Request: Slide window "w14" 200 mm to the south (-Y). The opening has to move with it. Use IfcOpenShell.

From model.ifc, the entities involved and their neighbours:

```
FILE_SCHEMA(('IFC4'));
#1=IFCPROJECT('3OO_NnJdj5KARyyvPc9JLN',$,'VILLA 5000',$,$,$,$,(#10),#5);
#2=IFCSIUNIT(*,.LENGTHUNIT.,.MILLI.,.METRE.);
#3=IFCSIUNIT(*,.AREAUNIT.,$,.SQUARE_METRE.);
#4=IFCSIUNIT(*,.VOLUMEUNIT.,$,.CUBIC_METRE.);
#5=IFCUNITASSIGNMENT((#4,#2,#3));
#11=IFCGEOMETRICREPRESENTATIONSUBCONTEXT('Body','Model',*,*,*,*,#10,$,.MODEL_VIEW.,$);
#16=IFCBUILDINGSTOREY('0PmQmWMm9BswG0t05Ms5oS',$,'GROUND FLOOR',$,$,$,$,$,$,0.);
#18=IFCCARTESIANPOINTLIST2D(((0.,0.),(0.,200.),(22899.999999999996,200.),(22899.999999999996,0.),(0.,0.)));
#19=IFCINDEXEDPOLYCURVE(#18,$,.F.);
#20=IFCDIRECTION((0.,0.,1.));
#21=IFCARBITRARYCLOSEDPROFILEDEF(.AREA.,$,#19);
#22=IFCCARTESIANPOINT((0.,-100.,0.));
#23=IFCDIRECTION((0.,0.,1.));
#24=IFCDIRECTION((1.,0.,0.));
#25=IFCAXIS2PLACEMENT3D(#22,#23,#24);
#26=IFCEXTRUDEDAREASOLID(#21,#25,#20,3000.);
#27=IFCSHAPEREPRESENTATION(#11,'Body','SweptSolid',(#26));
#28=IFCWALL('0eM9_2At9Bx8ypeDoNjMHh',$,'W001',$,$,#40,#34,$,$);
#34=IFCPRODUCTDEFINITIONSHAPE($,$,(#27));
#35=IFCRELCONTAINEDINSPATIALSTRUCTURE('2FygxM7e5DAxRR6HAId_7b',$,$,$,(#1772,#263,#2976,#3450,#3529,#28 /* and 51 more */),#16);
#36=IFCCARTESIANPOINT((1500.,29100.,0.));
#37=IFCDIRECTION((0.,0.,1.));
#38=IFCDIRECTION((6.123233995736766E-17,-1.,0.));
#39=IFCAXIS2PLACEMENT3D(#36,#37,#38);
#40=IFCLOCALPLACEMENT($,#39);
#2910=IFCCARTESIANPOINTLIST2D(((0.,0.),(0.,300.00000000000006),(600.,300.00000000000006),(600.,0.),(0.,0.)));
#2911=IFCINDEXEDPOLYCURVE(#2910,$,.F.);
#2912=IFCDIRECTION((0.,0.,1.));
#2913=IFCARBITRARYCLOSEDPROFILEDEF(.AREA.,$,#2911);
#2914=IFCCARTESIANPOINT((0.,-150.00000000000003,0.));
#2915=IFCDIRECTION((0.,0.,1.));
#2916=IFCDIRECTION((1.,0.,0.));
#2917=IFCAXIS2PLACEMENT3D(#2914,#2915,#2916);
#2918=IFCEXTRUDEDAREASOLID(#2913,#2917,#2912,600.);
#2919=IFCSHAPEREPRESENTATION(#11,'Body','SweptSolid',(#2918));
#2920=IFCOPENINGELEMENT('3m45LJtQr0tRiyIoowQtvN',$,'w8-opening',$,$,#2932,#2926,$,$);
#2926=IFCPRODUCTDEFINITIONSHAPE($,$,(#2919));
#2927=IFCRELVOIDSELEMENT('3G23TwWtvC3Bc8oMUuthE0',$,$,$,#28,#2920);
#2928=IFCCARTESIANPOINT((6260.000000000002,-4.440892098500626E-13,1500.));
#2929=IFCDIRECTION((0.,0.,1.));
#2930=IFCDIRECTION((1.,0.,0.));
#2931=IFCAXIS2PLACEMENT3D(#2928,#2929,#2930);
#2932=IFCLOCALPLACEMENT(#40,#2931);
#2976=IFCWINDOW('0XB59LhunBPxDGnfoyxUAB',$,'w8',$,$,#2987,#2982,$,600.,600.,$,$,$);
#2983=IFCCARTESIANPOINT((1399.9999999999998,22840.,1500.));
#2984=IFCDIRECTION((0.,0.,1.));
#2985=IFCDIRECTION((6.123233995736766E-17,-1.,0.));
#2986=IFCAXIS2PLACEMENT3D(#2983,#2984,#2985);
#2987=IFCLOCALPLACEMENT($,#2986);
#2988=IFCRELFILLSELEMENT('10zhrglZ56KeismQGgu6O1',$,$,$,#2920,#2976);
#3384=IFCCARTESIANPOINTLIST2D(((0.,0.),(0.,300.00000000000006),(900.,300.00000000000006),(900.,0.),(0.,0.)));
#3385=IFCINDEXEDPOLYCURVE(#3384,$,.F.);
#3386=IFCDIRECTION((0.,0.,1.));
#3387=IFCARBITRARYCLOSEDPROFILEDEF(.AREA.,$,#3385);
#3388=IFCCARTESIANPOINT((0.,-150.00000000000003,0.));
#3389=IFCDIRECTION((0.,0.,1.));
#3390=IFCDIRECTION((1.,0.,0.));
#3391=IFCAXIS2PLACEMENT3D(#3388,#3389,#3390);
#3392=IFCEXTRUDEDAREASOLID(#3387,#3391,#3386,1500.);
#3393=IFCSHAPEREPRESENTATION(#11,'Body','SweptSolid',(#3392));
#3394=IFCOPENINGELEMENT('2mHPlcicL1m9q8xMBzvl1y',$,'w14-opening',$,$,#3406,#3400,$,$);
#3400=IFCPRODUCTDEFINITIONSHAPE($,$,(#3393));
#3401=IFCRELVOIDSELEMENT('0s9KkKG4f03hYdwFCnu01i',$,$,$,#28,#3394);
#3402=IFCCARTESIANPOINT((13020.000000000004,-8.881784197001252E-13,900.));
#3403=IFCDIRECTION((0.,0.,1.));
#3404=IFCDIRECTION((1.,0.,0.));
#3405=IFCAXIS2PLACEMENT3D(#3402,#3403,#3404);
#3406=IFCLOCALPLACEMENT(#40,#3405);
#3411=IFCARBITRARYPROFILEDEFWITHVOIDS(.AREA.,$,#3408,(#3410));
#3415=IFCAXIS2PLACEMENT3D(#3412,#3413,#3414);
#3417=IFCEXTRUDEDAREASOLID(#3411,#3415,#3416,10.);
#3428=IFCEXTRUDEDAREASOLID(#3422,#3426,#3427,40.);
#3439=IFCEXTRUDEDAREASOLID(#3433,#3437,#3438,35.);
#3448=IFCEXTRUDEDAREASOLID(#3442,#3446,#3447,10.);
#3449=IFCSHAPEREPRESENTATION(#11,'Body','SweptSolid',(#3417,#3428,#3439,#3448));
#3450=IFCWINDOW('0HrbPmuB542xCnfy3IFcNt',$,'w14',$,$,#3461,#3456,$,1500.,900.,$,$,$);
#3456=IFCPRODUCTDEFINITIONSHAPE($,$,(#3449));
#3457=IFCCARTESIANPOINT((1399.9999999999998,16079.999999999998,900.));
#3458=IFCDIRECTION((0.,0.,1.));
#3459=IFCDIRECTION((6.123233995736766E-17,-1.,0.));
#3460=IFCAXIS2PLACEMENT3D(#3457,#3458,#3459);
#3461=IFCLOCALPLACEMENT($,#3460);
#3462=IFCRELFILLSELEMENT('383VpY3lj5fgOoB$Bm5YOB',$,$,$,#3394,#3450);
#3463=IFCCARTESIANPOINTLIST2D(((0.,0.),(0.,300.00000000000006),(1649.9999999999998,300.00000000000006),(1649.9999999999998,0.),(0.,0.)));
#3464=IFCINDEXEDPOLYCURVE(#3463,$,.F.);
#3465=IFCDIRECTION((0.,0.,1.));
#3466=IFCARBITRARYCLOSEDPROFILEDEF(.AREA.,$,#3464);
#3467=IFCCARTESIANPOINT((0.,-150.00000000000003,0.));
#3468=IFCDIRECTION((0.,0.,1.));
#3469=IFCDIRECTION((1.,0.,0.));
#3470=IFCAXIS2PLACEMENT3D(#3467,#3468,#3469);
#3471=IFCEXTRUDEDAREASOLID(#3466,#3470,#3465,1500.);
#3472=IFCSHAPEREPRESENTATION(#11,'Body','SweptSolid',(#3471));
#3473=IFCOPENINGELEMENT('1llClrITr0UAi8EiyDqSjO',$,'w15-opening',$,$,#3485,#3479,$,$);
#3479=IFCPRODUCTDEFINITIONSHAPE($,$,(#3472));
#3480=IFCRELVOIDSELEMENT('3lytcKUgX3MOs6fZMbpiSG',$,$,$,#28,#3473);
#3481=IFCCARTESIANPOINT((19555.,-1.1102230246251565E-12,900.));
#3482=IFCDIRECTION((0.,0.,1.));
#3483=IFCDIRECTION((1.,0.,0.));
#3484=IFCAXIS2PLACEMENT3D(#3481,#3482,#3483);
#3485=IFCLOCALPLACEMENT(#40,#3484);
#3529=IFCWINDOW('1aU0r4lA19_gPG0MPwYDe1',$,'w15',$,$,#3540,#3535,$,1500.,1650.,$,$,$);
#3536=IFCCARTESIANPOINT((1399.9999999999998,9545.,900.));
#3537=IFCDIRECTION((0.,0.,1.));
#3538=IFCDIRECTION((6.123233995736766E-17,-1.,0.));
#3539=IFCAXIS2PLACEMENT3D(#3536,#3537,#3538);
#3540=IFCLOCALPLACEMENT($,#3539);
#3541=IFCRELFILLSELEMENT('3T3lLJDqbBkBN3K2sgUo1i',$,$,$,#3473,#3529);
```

```python
import ifcopenshell
import ifcopenshell.api.geometry
import ifcopenshell.util.placement

model = ifcopenshell.open("model.ifc")

window = model.by_id(3450)
opening = window.FillsVoids[0].RelatingOpeningElement
wall = opening.VoidsElements[0].RelatingBuildingElement

wall_matrix = ifcopenshell.util.placement.get_local_placement(wall.ObjectPlacement)
shift = wall_matrix[:3, 0] * 200.0
before = ifcopenshell.util.placement.get_local_placement(window.ObjectPlacement)[:3, 3].copy()

# The window is not placed relative to its opening, so move both.
for product in (opening, window):
    matrix = ifcopenshell.util.placement.get_local_placement(product.ObjectPlacement)
    matrix[:3, 3] += shift
    ifcopenshell.api.geometry.edit_object_placement(model, product=product, matrix=matrix, is_si=False)

after = ifcopenshell.util.placement.get_local_placement(window.ObjectPlacement)[:3, 3]
print("window moved by", (after - before).round(3) + 0.0)

model.write("model_rev.ifc")
```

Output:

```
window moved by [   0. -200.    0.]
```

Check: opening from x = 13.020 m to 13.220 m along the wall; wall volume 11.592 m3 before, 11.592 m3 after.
